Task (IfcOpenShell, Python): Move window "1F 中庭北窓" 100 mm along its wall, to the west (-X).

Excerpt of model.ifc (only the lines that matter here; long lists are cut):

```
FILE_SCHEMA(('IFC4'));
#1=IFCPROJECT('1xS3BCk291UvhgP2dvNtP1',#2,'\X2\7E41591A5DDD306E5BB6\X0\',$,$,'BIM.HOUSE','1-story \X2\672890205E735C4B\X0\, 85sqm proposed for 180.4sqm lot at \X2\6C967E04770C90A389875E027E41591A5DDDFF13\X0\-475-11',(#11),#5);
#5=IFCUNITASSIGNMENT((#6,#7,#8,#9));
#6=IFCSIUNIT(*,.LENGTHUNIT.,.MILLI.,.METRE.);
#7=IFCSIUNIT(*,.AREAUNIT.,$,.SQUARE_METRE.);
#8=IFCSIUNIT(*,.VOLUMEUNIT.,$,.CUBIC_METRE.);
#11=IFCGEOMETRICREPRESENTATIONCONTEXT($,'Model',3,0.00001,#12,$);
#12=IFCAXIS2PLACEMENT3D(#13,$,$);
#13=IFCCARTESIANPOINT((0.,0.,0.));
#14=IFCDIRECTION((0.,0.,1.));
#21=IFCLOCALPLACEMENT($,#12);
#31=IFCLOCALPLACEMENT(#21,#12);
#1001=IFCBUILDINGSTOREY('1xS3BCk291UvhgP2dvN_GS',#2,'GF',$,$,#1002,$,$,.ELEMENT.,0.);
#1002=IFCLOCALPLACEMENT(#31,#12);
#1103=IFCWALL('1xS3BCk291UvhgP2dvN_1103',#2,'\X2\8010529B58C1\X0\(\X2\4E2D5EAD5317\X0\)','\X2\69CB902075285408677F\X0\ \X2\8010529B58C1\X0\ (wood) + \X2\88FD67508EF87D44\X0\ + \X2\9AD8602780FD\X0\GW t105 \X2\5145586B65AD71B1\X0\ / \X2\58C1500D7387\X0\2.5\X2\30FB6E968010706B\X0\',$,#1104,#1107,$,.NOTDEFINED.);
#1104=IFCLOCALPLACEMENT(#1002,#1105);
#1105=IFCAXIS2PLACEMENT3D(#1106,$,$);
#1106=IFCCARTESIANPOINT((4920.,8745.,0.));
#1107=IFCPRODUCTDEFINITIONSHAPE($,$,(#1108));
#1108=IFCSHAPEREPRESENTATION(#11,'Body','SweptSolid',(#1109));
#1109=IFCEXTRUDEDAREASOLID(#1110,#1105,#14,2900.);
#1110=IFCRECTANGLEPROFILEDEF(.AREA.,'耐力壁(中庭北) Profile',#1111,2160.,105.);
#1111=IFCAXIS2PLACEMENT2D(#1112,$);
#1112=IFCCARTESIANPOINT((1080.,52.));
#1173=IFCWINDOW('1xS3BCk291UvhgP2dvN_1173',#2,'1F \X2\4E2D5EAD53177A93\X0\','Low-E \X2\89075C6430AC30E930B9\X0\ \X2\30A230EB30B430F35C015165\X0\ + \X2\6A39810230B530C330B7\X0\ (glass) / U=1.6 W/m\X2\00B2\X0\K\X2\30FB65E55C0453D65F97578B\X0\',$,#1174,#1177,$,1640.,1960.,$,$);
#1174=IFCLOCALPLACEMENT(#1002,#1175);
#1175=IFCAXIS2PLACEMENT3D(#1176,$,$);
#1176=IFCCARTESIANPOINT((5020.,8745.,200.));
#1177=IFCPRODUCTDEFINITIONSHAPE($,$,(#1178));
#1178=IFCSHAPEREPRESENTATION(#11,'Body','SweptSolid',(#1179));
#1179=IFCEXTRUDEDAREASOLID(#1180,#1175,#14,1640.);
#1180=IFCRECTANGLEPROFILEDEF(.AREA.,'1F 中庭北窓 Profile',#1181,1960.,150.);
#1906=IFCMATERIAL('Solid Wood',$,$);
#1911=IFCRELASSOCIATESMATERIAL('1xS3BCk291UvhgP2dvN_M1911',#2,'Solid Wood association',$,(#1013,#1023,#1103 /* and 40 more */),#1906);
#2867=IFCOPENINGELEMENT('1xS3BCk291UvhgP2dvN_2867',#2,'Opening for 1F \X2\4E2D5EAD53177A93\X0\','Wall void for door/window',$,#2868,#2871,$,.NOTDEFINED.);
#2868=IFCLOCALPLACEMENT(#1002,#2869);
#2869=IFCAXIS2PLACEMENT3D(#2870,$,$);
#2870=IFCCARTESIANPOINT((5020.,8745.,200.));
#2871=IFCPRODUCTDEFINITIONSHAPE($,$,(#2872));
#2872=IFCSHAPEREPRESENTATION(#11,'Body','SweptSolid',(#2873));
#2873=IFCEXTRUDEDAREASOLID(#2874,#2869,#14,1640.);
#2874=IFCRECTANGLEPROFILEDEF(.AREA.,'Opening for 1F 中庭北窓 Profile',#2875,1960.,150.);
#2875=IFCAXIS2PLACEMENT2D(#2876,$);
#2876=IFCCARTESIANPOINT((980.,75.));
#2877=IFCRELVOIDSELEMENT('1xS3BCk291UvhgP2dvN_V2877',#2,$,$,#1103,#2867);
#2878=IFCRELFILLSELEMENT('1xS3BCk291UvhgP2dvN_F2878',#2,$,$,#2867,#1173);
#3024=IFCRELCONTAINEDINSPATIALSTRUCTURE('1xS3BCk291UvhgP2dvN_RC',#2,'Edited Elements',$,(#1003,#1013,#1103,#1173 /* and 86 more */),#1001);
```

```python
import ifcopenshell
import ifcopenshell.api.geometry
import ifcopenshell.util.placement

model = ifcopenshell.open("model.ifc")

window = model.by_guid("1xS3BCk291UvhgP2dvN_1173")
opening = window.FillsVoids[0].RelatingOpeningElement
wall = opening.VoidsElements[0].RelatingBuildingElement

wall_matrix = ifcopenshell.util.placement.get_local_placement(wall.ObjectPlacement)
shift = wall_matrix[:3, 0] * -100.0
before = ifcopenshell.util.placement.get_local_placement(window.ObjectPlacement)[:3, 3].copy()

# The window is not placed relative to its opening, so move both.
for product in (opening, window):
    matrix = ifcopenshell.util.placement.get_local_placement(product.ObjectPlacement)
    matrix[:3, 3] += shift
    ifcopenshell.api.geometry.edit_object_placement(model, product=product, matrix=matrix, is_si=False)

after = ifcopenshell.util.placement.get_local_placement(window.ObjectPlacement)[:3, 3]
print("window moved by", (after - before).round(3) + 0.0)

model.write("model_edited.ifc")
```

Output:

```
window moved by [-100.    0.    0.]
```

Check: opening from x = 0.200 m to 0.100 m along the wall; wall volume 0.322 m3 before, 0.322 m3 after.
